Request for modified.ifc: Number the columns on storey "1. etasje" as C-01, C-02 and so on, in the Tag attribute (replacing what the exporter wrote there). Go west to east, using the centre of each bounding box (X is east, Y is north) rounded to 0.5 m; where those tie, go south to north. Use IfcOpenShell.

First a look at what the model holds.

```python
import ifcopenshell
import ifcopenshell.util.element
import ifcopenshell.util.placement

model = ifcopenshell.open("modified.ifc")
print(model.schema)
storey = next(s for s in model.by_type("IfcBuildingStorey") if s.Name == "1. etasje")
columns = [e for e in ifcopenshell.util.element.get_decomposition(storey) if e.is_a("IfcColumn")]
for e in sorted(columns, key=lambda e: e.id()):
    origin = ifcopenshell.util.placement.get_local_placement(e.ObjectPlacement)[:3, 3]
    print(e.id(), e.Tag, e.Name, origin.round(2) + 0.0, sep=" | ")
```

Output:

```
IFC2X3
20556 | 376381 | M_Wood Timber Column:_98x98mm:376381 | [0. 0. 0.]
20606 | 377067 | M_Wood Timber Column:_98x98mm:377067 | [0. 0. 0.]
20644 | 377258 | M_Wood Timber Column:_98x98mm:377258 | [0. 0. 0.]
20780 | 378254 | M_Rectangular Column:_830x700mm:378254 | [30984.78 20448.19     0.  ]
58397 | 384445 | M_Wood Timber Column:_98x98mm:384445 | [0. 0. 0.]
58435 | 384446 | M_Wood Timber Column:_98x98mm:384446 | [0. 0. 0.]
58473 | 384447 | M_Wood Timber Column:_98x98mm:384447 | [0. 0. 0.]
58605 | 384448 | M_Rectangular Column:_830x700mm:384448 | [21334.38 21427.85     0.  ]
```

```python
import ifcopenshell
import ifcopenshell.geom
import ifcopenshell.util.element
import ifcopenshell.util.shape

model = ifcopenshell.open("modified.ifc")
settings = ifcopenshell.geom.settings()
settings.set("use-world-coords", True)


def centre(element):
    shape = ifcopenshell.geom.create_shape(settings, element)
    return ifcopenshell.util.shape.get_bbox_centroid(shape.geometry)


storey = next(s for s in model.by_type("IfcBuildingStorey") if s.Name == "1. etasje")
columns = [e for e in ifcopenshell.util.element.get_decomposition(storey) if e.is_a("IfcColumn")]

# Insertion points can sit at a corner or the storey origin, so sort by the geometry (in metres).
centres = {e: centre(e) for e in columns}
columns.sort(key=lambda e: (round(centres[e][0] / 0.5), centres[e][1]))

for i, e in enumerate(columns, start=1):
    number = f"C-{i:02d}"
    e.Tag = number
    print(e.id(), number)

model.write("modified_rev.ifc")
```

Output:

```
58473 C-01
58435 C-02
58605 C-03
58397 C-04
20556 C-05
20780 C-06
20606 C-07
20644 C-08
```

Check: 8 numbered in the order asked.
